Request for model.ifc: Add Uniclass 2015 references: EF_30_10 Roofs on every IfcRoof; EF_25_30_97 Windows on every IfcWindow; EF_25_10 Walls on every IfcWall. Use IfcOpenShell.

First a look at what the model holds.

```python
import ifcopenshell

model = ifcopenshell.open("model.ifc")
print(model.schema)
print("classifications:", [c.Name for c in model.by_type("IfcClassification")])
for ifc_class in ("IfcDoor", "IfcRoof", "IfcStair", "IfcWall", "IfcWindow"):
    print(ifc_class, len(model.by_type(ifc_class)))
```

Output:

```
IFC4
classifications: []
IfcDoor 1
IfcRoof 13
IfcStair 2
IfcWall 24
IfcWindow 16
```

```python
import ifcopenshell
import ifcopenshell.api.classification

model = ifcopenshell.open("model.ifc")

system = ifcopenshell.api.classification.add_classification(model, classification="Uniclass 2015")

codes = {
    "IfcRoof": ("EF_30_10", "Roofs"),
    "IfcWindow": ("EF_25_30_97", "Windows"),
    "IfcWall": ("EF_25_10", "Walls"),
}
for ifc_class, (code, name) in codes.items():
    products = model.by_type(ifc_class)
    ifcopenshell.api.classification.add_reference(
        model, products=products, classification=system, identification=code, name=name
    )
    print(code, len(products))

model.write("model-out.ifc")
```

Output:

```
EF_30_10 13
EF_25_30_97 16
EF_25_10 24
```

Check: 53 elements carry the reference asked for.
